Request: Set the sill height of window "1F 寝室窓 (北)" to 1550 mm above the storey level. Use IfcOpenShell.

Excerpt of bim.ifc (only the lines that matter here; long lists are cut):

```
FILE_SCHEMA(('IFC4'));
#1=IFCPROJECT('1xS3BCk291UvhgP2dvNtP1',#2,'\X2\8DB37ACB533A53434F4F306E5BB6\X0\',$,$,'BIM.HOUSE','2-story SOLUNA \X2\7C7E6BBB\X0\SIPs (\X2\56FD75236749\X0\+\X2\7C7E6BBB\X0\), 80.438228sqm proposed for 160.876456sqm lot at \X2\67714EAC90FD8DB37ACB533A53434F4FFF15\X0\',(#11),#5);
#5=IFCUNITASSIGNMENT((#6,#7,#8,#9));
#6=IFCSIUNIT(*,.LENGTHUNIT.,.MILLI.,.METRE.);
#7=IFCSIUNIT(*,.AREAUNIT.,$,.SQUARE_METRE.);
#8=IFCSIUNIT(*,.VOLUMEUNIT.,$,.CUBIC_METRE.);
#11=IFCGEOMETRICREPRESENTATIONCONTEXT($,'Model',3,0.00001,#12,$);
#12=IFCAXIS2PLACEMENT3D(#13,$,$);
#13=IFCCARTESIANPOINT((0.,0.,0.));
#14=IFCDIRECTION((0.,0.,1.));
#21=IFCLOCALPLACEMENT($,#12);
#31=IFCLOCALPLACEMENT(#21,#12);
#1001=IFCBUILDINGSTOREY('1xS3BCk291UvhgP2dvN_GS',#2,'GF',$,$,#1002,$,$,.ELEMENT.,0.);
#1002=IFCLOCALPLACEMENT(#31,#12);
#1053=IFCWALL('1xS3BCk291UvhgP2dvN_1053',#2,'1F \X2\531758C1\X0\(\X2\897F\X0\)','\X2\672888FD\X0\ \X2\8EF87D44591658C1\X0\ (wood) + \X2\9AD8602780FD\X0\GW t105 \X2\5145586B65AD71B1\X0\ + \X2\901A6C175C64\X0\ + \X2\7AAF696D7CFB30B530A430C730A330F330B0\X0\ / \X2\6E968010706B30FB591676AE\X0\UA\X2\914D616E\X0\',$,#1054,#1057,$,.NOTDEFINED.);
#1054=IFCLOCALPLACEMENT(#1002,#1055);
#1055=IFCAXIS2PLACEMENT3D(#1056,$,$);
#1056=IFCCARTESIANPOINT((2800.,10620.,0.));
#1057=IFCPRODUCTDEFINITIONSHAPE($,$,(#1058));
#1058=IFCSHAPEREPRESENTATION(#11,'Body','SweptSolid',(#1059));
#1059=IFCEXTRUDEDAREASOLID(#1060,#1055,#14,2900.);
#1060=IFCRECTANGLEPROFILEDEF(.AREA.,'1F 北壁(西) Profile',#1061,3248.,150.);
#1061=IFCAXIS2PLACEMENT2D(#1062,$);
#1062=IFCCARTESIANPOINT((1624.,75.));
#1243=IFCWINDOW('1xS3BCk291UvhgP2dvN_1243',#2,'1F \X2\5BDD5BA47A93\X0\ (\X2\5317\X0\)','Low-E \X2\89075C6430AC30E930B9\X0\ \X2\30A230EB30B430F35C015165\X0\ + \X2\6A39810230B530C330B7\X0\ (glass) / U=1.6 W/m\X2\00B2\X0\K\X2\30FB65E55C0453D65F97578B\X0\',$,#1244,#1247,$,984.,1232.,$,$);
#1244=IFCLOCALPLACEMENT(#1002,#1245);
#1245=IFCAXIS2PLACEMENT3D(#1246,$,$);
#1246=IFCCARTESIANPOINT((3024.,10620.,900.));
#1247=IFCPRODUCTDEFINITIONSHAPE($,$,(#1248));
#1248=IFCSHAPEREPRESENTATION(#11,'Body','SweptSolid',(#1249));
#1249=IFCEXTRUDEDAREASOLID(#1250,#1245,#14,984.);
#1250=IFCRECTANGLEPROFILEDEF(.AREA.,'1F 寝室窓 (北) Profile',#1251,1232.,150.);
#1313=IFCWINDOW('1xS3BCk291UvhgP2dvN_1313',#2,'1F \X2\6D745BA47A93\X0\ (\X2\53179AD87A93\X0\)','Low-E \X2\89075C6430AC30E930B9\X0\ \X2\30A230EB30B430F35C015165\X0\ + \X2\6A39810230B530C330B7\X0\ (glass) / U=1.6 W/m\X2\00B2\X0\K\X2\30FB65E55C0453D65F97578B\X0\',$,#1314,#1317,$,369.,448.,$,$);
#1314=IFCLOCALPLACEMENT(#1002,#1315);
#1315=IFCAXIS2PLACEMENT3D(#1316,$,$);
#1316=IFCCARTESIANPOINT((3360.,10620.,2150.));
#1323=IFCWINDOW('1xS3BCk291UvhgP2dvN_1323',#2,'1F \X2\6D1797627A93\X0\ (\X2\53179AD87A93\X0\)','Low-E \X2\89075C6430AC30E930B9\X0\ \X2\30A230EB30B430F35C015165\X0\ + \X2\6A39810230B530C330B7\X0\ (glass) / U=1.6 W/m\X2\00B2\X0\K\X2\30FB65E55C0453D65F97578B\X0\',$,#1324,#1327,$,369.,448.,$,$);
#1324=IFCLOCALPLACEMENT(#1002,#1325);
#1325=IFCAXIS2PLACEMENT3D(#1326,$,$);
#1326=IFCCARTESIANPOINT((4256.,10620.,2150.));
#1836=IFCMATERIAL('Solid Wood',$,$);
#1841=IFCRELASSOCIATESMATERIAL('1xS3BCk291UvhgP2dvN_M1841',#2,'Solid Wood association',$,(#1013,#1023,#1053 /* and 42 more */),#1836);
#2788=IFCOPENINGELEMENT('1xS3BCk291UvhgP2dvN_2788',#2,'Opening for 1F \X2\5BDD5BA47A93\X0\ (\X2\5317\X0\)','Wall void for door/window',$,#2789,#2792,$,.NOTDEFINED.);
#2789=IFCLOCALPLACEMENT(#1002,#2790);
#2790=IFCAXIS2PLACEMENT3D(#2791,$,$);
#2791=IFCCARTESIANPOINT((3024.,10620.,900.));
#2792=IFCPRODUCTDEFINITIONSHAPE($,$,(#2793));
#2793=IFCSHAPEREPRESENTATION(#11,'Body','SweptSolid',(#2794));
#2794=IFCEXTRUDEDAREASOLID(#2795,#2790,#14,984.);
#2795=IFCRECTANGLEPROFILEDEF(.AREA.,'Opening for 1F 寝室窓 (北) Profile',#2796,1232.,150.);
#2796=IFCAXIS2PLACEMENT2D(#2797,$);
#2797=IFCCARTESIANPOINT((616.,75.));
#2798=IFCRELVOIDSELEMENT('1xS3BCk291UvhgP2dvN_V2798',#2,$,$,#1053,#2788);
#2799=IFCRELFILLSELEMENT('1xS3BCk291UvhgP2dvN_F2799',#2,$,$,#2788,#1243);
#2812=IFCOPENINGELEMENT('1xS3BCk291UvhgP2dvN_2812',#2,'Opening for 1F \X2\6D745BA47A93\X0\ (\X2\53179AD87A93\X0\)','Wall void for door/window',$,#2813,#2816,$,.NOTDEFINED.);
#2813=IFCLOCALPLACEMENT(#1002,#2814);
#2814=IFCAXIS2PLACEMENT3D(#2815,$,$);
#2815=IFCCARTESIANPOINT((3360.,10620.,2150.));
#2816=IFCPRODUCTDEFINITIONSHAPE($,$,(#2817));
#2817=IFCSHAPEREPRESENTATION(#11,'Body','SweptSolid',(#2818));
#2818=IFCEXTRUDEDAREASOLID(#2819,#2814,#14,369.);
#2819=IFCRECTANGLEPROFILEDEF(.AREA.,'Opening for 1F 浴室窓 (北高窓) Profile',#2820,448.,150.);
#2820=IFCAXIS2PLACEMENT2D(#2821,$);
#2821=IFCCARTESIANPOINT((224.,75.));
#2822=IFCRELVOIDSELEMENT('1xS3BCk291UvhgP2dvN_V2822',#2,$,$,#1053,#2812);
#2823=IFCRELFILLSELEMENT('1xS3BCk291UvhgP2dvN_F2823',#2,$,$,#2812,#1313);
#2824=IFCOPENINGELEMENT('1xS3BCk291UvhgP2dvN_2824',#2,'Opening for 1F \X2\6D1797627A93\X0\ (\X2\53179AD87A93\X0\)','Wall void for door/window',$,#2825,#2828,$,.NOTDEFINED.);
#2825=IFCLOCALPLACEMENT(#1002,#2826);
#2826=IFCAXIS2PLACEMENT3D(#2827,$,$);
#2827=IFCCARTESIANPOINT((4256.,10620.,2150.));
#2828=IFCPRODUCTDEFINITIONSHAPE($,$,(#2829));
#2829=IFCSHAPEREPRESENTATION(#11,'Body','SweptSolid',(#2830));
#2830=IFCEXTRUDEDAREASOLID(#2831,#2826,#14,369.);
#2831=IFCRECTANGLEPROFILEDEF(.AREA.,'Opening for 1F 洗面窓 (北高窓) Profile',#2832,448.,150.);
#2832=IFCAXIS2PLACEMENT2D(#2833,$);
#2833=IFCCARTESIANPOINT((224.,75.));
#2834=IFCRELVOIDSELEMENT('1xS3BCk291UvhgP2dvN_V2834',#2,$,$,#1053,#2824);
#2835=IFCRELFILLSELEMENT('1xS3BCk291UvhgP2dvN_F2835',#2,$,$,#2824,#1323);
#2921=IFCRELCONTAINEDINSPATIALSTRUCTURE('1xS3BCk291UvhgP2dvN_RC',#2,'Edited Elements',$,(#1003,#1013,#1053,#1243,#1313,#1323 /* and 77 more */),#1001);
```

```python
import numpy as np
import ifcopenshell
import ifcopenshell.api.geometry
import ifcopenshell.geom
import ifcopenshell.util.element
import ifcopenshell.util.placement
import ifcopenshell.util.shape
import ifcopenshell.util.unit

model = ifcopenshell.open("bim.ifc")
unit_scale = ifcopenshell.util.unit.calculate_unit_scale(model)

window = model.by_guid("1xS3BCk291UvhgP2dvN_1243")
opening = window.FillsVoids[0].RelatingOpeningElement
storey = ifcopenshell.util.element.get_container(window, ifc_class="IfcBuildingStorey")
level = ifcopenshell.util.placement.get_local_placement(storey.ObjectPlacement)[2, 3]

# The opening's origin need not be at the sill, so measure its lowest point.
shape = ifcopenshell.geom.create_shape(ifcopenshell.geom.settings(), opening)
bottom = ifcopenshell.util.shape.get_shape_bottom_elevation(shape, shape.geometry) / unit_scale
dz = level + 1550.0 - bottom

shift = np.array([0.0, 0.0, dz])
# The window is not placed relative to its opening, so move both.
for product in (opening, window):
    matrix = ifcopenshell.util.placement.get_local_placement(product.ObjectPlacement)
    matrix[:3, 3] += shift
    ifcopenshell.api.geometry.edit_object_placement(model, product=product, matrix=matrix, is_si=False)

print(f"moved by {dz * unit_scale:+.3f} m")

model.write("bim_edited.ifc")
```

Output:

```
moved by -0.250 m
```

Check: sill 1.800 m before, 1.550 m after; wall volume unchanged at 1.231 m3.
